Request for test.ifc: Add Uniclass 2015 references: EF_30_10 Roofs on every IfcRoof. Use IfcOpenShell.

First a look at what the model holds.

```python
import ifcopenshell

model = ifcopenshell.open("test.ifc")
print(model.schema)
print("classifications:", [c.Name for c in model.by_type("IfcClassification")])
for ifc_class in ("IfcDoor", "IfcRoof", "IfcStair", "IfcWall", "IfcWindow"):
    print(ifc_class, len(model.by_type(ifc_class)))
```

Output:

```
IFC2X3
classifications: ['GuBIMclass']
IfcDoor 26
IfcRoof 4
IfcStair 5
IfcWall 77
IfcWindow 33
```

```python
import ifcopenshell
import ifcopenshell.api.classification

model = ifcopenshell.open("test.ifc")

# IFC2X3 requires Source and Edition and has no link from the project to the system.
system = model.create_entity("IfcClassification", Source="NBS", Edition="2015", Name="Uniclass 2015")

codes = {
    "IfcRoof": ("EF_30_10", "Roofs"),
}
for ifc_class, (code, name) in codes.items():
    products = model.by_type(ifc_class)
    ifcopenshell.api.classification.add_reference(
        model, products=products, classification=system, identification=code, name=name
    )
    print(code, len(products))

model.write("test_edited.ifc")
```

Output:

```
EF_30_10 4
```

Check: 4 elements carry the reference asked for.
